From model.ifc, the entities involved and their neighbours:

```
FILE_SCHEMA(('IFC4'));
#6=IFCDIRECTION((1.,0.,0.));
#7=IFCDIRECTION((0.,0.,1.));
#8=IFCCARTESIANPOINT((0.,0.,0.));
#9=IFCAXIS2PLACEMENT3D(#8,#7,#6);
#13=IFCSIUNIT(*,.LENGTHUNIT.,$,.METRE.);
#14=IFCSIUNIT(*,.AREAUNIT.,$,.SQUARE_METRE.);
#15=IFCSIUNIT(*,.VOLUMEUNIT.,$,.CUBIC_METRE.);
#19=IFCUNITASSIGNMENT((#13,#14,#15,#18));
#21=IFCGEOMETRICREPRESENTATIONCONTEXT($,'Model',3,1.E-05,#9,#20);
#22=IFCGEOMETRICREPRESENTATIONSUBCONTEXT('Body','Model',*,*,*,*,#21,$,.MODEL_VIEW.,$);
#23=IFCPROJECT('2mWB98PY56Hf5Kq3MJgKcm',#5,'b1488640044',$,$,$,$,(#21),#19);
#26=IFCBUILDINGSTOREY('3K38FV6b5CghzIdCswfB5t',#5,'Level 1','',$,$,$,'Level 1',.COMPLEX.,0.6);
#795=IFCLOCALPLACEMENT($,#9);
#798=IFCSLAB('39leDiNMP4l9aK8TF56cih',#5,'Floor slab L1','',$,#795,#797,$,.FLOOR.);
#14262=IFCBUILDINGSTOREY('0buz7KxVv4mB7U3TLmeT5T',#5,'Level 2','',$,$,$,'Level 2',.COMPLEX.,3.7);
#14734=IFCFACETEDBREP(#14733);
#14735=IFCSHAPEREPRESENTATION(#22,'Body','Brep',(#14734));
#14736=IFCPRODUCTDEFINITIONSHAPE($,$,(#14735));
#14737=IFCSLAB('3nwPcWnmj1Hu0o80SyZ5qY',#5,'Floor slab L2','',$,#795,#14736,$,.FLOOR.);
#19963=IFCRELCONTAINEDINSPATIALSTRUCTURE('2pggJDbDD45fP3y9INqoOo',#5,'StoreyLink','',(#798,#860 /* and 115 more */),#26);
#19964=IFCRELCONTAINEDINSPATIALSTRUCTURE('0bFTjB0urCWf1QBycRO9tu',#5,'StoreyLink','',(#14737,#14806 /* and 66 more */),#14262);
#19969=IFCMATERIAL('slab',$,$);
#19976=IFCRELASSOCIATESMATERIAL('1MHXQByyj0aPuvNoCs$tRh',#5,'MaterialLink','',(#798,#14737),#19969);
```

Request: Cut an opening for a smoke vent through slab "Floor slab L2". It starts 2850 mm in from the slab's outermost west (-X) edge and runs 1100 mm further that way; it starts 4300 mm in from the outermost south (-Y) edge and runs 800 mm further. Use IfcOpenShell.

```python
import numpy as np
import ifcopenshell
import ifcopenshell.api.feature
import ifcopenshell.api.geometry
import ifcopenshell.api.root
import ifcopenshell.geom
import ifcopenshell.util.placement
import ifcopenshell.util.representation
import ifcopenshell.util.shape
import ifcopenshell.util.unit

model = ifcopenshell.open("model.ifc")
unit_scale = ifcopenshell.util.unit.calculate_unit_scale(model)
settings = ifcopenshell.geom.settings()


def volume(element):
    """Net volume in cubic metres, openings subtracted."""
    shape = ifcopenshell.geom.create_shape(settings, element)
    return ifcopenshell.util.shape.get_volume(shape.geometry)


slab = model.by_id(14737)
before = volume(slab)

# Extent in the slab's own axes, in metres. The edges named are its -X and -Y sides.
slab_shape = ifcopenshell.geom.create_shape(settings, slab)
vertices = ifcopenshell.util.shape.get_vertices(slab_shape.geometry)
x_min, y_min, bottom = vertices.min(axis=0)
top = vertices[:, 2].max()

opening = ifcopenshell.api.root.create_entity(model, ifc_class="IfcOpeningElement", name="Smoke vent opening", predefined_type="OPENING")
context = ifcopenshell.util.representation.get_context(model, "Model", "Body", "MODEL_VIEW")
width, depth = 1.1, 0.8
outline = [(0.0, 0.0), (width, 0.0), (width, depth), (0.0, depth), (0.0, 0.0)]
# Overshoot both faces by 50 mm so the cut is clean.
shape = ifcopenshell.api.geometry.add_slab_representation(
    model, context=context, depth=top - bottom + 0.1, polyline=outline
)
ifcopenshell.api.geometry.assign_representation(model, product=opening, representation=shape)

matrix = ifcopenshell.util.placement.get_local_placement(slab.ObjectPlacement)
matrix[:, 3] = matrix @ np.append(np.array([x_min + 2.85, y_min + 4.3, bottom - 0.05]) / unit_scale, 1.0)
ifcopenshell.api.geometry.edit_object_placement(model, product=opening, matrix=matrix, is_si=False)
ifcopenshell.api.feature.add_feature(model, feature=opening, element=slab)

after = volume(slab)

print(f"slab volume {before:.3f} -> {after:.3f} m3")

model.write("model_rev.ifc")
```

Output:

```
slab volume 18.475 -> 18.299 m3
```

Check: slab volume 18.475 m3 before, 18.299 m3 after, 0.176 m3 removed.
